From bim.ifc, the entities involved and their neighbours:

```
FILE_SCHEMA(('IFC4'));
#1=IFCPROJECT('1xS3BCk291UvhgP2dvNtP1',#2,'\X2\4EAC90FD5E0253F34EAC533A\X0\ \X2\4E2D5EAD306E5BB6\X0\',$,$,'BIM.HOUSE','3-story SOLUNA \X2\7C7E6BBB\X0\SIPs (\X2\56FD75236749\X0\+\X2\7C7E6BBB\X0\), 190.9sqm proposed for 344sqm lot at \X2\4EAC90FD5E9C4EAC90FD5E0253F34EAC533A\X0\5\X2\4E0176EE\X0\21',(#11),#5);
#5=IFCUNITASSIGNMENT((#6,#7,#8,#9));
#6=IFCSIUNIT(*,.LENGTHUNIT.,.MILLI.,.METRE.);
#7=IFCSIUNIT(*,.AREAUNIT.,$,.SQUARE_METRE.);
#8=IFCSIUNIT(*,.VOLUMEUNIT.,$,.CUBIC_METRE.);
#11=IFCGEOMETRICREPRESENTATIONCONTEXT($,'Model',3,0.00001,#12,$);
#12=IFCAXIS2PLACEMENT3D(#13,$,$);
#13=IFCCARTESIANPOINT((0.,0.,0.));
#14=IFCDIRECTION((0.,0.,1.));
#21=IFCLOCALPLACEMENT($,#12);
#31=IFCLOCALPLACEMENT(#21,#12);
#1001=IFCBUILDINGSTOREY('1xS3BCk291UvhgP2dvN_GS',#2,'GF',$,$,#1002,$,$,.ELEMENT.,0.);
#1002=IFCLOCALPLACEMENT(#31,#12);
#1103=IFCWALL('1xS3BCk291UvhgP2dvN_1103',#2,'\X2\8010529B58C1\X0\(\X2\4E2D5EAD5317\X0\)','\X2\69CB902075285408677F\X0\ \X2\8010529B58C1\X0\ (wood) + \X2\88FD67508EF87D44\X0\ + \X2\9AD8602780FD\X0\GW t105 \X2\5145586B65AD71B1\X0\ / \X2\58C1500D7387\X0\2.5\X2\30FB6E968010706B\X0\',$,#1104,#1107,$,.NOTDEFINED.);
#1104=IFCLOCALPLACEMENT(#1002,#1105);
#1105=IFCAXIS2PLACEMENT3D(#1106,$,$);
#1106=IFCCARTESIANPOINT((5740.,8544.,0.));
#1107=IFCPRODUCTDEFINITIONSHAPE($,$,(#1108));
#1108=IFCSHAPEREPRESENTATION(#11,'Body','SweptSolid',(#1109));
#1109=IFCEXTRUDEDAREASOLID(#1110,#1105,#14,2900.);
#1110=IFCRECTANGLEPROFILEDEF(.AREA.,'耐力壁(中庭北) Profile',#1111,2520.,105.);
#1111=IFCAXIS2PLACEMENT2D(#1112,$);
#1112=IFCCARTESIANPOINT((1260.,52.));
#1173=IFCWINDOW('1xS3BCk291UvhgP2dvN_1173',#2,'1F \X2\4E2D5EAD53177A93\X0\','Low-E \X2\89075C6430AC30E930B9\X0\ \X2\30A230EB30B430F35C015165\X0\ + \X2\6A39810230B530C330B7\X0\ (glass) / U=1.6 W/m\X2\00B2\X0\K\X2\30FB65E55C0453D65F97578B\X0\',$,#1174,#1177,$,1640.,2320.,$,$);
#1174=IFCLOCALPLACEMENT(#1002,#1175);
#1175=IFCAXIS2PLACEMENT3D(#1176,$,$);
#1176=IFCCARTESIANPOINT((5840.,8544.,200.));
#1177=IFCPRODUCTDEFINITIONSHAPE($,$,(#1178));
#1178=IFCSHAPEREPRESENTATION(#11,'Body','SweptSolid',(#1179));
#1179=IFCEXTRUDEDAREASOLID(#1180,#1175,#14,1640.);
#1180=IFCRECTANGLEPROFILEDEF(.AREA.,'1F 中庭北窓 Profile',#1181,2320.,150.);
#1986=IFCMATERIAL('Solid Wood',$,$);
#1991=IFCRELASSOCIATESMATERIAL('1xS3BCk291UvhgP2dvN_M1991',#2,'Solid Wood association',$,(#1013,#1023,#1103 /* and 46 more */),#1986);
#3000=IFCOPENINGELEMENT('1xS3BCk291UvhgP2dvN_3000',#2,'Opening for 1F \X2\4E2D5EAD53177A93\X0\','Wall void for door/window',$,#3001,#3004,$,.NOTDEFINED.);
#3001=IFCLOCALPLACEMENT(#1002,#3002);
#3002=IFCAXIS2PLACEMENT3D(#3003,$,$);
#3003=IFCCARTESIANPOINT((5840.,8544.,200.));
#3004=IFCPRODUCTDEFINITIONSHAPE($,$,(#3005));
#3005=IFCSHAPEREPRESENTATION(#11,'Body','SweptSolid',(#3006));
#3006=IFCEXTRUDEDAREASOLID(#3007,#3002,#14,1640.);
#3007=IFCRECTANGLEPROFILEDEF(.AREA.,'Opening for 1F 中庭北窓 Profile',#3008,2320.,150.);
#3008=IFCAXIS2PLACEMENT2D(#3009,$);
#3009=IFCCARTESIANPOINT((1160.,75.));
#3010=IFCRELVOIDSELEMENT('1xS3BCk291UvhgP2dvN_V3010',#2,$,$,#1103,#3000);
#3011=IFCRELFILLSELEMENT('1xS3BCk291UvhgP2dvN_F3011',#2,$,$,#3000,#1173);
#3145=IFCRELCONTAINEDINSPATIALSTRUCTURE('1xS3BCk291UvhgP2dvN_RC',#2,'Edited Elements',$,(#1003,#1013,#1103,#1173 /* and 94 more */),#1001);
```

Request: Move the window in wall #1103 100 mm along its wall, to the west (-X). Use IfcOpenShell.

```python
import ifcopenshell
import ifcopenshell.api.geometry
import ifcopenshell.util.placement
import ifcopenshell.util.unit

model = ifcopenshell.open("bim.ifc")
unit_scale = ifcopenshell.util.unit.calculate_unit_scale(model)

window = model.by_guid("1xS3BCk291UvhgP2dvN_1173")
opening = window.FillsVoids[0].RelatingOpeningElement
wall = opening.VoidsElements[0].RelatingBuildingElement

wall_matrix = ifcopenshell.util.placement.get_local_placement(wall.ObjectPlacement)
shift = wall_matrix[:3, 0] * -0.1 / unit_scale
before = ifcopenshell.util.placement.get_local_placement(window.ObjectPlacement)[:3, 3].copy()

# The window is not placed relative to its opening, so move both.
for product in (opening, window):
    matrix = ifcopenshell.util.placement.get_local_placement(product.ObjectPlacement)
    matrix[:3, 3] += shift
    ifcopenshell.api.geometry.edit_object_placement(model, product=product, matrix=matrix, is_si=False)

after = ifcopenshell.util.placement.get_local_placement(window.ObjectPlacement)[:3, 3]
print("window moved by", (after - before).round(3) + 0.0)

model.write("bim_edited.ifc")
```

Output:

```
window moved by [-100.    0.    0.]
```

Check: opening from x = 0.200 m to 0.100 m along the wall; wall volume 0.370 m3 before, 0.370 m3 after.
